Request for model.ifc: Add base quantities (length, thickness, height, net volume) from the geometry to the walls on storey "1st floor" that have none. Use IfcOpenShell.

First a look at what the model holds.

```python
import ifcopenshell
import ifcopenshell.util.element
import ifcopenshell.util.unit

model = ifcopenshell.open("model.ifc")
print(model.schema)
for unit_type in ("LENGTHUNIT", "AREAUNIT", "VOLUMEUNIT"):
    print(unit_type, ifcopenshell.util.unit.calculate_unit_scale(model, unit_type))
storey = next(s for s in model.by_type("IfcBuildingStorey") if s.Name == "1st floor")
walls = [e for e in ifcopenshell.util.element.get_decomposition(storey) if e.is_a("IfcWall")]
for e in sorted(walls, key=lambda e: e.id()):
    print(e.id(), e.is_a(), e.Name, list(ifcopenshell.util.element.get_psets(e, qtos_only=True)), sep=" | ")
```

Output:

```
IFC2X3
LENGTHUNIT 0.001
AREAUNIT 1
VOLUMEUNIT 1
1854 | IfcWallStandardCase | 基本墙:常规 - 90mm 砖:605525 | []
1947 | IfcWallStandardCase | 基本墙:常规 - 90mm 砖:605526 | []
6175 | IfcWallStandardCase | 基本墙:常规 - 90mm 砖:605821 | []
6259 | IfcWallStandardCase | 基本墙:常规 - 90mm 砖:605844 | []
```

```python
import ifcopenshell
import ifcopenshell.api.pset
import ifcopenshell.geom
import ifcopenshell.util.element
import ifcopenshell.util.shape
import ifcopenshell.util.unit

model = ifcopenshell.open("model.ifc")
unit_scale = ifcopenshell.util.unit.calculate_unit_scale(model)
volume_scale = ifcopenshell.util.unit.calculate_unit_scale(model, "VOLUMEUNIT")
settings = ifcopenshell.geom.settings()

storey = next(s for s in model.by_type("IfcBuildingStorey") if s.Name == "1st floor")
walls = [e for e in ifcopenshell.util.element.get_decomposition(storey) if e.is_a("IfcWall")]

for e in sorted(walls, key=lambda e: e.id()):
    if ifcopenshell.util.element.get_psets(e, qtos_only=True, should_inherit=False):
        continue
    # Geometry comes back in metres, in the element's own axes.
    shape = ifcopenshell.geom.create_shape(settings, e)
    values = {
        "Length": ifcopenshell.util.shape.get_x(shape.geometry) / unit_scale,
        "Width": ifcopenshell.util.shape.get_y(shape.geometry) / unit_scale,
        "Height": ifcopenshell.util.shape.get_z(shape.geometry) / unit_scale,
        "NetVolume": ifcopenshell.util.shape.get_volume(shape.geometry) / volume_scale,
    }
    qto = ifcopenshell.api.pset.add_qto(model, product=e, name="BaseQuantities")
    ifcopenshell.api.pset.edit_qto(model, qto=qto, properties=values)
    print(e.id(), {k: round(v, 3) for k, v in values.items()})

model.write("model_rev.ifc")
```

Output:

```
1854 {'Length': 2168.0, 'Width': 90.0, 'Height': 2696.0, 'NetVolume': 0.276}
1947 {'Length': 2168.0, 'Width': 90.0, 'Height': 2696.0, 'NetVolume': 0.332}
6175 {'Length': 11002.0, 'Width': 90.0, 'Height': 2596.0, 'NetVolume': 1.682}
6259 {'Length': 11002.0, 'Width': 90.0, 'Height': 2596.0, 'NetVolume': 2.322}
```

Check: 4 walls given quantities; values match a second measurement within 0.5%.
